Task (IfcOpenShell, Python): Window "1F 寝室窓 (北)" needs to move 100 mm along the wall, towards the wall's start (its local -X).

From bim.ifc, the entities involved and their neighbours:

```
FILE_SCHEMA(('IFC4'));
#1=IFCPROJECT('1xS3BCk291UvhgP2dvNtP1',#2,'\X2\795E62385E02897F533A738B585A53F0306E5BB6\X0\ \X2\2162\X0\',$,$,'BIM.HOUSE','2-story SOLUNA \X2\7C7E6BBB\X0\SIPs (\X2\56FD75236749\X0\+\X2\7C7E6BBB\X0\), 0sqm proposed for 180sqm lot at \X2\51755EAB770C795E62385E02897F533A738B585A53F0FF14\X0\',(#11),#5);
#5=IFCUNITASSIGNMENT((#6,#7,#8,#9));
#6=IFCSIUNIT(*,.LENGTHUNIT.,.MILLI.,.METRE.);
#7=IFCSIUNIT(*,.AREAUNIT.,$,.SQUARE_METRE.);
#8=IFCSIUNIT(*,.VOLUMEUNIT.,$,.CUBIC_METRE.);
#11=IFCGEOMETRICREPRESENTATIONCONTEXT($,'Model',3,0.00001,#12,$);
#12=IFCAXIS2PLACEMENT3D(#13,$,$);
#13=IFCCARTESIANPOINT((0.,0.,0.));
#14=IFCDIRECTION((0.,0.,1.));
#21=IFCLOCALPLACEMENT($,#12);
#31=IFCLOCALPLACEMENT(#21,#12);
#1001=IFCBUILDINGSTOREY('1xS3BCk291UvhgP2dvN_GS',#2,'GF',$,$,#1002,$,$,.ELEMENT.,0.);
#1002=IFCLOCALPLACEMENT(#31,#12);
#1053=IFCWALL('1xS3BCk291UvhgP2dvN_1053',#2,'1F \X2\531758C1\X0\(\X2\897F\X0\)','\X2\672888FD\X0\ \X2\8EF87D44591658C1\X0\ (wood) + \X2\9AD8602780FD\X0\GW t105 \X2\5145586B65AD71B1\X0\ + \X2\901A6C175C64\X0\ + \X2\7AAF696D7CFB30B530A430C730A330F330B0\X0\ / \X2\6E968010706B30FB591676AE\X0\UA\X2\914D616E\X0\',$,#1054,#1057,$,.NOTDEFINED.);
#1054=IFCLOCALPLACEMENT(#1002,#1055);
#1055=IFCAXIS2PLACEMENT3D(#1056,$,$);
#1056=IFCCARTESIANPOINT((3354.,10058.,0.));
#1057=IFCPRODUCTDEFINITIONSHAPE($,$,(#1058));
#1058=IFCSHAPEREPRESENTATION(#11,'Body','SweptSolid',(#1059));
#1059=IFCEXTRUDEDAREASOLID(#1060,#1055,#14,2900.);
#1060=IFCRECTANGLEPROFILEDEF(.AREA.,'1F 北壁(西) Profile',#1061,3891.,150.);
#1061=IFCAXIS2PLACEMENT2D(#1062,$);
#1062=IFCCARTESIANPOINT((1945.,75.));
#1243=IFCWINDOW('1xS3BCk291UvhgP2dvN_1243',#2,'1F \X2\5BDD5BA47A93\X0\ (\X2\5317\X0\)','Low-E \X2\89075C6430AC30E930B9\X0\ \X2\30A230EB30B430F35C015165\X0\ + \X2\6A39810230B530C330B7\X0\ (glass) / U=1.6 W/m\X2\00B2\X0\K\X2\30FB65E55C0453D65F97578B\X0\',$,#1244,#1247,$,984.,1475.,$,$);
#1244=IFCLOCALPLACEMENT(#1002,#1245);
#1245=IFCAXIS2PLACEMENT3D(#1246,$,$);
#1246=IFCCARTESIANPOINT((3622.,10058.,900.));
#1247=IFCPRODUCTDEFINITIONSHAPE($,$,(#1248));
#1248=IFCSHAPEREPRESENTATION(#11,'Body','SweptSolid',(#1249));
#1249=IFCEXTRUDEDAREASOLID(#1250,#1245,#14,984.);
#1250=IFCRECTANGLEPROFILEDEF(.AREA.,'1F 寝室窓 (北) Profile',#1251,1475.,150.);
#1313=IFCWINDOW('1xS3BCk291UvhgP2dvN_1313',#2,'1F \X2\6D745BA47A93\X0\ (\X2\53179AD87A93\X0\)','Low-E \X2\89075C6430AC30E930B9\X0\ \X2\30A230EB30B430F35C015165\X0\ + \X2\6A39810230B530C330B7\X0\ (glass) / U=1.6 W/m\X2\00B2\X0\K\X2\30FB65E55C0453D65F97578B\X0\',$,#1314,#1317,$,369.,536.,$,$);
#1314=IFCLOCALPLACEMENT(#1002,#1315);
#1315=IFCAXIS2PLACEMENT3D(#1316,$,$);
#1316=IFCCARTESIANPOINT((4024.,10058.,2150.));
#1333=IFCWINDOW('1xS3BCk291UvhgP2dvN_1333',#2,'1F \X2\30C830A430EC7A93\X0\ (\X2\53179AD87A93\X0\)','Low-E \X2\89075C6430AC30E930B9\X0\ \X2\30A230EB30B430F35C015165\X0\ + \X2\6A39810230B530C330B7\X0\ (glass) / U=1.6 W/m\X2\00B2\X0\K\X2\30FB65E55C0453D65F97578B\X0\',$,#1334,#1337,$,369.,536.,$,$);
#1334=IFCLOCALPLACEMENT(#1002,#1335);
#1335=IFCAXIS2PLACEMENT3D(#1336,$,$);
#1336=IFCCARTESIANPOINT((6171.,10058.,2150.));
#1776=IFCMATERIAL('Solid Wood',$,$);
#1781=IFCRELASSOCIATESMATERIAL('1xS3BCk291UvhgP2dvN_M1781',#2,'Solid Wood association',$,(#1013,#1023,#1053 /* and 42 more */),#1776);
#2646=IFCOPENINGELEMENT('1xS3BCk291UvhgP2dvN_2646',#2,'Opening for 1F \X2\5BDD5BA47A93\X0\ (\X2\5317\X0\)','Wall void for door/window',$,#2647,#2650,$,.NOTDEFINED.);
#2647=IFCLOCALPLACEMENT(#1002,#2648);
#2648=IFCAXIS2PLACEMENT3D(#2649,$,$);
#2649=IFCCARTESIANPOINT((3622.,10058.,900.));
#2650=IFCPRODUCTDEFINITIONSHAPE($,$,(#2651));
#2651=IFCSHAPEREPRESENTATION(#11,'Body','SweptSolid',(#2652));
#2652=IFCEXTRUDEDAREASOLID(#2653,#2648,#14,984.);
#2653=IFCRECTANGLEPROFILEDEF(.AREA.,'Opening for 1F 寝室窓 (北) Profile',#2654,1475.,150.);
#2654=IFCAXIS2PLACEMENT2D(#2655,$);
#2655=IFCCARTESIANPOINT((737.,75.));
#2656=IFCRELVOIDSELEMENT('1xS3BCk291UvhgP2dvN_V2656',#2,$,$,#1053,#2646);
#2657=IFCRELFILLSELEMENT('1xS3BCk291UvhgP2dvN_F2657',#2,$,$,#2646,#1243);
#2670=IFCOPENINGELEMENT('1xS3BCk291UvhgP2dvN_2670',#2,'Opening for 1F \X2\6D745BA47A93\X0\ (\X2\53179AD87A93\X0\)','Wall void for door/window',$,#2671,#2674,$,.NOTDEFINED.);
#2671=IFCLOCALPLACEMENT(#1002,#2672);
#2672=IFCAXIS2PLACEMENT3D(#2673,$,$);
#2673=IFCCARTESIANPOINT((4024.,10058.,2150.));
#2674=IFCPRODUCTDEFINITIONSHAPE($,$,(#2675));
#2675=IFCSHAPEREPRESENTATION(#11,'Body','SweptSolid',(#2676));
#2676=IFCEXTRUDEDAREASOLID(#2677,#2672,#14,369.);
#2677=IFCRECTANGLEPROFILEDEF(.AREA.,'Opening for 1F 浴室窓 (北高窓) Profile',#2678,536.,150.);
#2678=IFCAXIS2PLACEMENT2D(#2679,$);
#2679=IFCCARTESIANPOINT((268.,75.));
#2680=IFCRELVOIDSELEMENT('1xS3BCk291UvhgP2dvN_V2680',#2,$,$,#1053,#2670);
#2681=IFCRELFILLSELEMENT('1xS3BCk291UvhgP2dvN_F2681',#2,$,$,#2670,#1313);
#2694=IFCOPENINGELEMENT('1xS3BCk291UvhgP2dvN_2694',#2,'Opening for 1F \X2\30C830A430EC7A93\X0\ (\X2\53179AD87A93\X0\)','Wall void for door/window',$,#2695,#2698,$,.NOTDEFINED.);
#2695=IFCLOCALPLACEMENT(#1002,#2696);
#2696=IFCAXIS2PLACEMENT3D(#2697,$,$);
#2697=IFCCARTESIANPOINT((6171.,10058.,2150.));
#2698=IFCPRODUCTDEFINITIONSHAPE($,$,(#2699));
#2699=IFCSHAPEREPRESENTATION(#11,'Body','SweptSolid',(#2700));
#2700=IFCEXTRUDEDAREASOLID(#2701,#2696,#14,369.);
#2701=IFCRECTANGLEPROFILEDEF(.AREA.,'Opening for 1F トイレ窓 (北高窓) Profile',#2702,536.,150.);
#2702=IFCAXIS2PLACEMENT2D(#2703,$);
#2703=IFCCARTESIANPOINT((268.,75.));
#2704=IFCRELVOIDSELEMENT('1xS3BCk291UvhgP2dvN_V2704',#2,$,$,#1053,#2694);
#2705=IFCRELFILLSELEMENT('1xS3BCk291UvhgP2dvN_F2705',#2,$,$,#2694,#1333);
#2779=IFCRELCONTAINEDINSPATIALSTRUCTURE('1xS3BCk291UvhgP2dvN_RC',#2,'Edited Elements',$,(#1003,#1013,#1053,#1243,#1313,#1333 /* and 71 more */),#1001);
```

```python
import ifcopenshell
import ifcopenshell.api.geometry
import ifcopenshell.util.placement

model = ifcopenshell.open("bim.ifc")

window = model.by_guid("1xS3BCk291UvhgP2dvN_1243")
opening = window.FillsVoids[0].RelatingOpeningElement
wall = opening.VoidsElements[0].RelatingBuildingElement

wall_matrix = ifcopenshell.util.placement.get_local_placement(wall.ObjectPlacement)
shift = wall_matrix[:3, 0] * -100.0
before = ifcopenshell.util.placement.get_local_placement(window.ObjectPlacement)[:3, 3].copy()

# The window is not placed relative to its opening, so move both.
for product in (opening, window):
    matrix = ifcopenshell.util.placement.get_local_placement(product.ObjectPlacement)
    matrix[:3, 3] += shift
    ifcopenshell.api.geometry.edit_object_placement(model, product=product, matrix=matrix, is_si=False)

after = ifcopenshell.util.placement.get_local_placement(window.ObjectPlacement)[:3, 3]
print("window moved by", (after - before).round(3) + 0.0)

model.write("bim_edited.ifc")
```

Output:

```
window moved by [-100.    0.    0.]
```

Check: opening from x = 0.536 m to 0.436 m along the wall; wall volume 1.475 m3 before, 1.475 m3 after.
